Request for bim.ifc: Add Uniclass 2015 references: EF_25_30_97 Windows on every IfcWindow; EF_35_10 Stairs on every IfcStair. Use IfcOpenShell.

First a look at what the model holds.

```python
import ifcopenshell

model = ifcopenshell.open("bim.ifc")
print(model.schema)
print("classifications:", [c.Name for c in model.by_type("IfcClassification")])
for ifc_class in ("IfcDoor", "IfcRoof", "IfcStair", "IfcWall", "IfcWindow"):
    print(ifc_class, len(model.by_type(ifc_class)))
```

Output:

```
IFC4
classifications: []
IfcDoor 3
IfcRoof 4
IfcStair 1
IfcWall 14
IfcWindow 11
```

```python
import ifcopenshell
import ifcopenshell.api.classification

model = ifcopenshell.open("bim.ifc")

system = ifcopenshell.api.classification.add_classification(model, classification="Uniclass 2015")

codes = {
    "IfcWindow": ("EF_25_30_97", "Windows"),
    "IfcStair": ("EF_35_10", "Stairs"),
}
for ifc_class, (code, name) in codes.items():
    products = model.by_type(ifc_class)
    ifcopenshell.api.classification.add_reference(
        model, products=products, classification=system, identification=code, name=name
    )
    print(code, len(products))

model.write("bim_edited.ifc")
```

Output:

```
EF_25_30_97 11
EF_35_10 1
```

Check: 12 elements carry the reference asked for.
